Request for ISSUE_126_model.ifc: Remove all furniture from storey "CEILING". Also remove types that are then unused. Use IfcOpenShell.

First a look at what the model holds.

```python
import ifcopenshell
import ifcopenshell.util.element

model = ifcopenshell.open("ISSUE_126_model.ifc")
print(model.schema)
storey = next(s for s in model.by_type("IfcBuildingStorey") if s.Name == "CEILING")
furniture = [e for e in ifcopenshell.util.element.get_decomposition(storey) if e.is_a("IfcFurnishingElement")]
seen = {}
for e in furniture:
    element_type = ifcopenshell.util.element.get_type(e)
    name = element_type.Name if element_type not in (None, e) else None
    seen[name] = seen.get(name, 0) + 1
for name, count in sorted(seen.items(), key=str):
    print(count, "x", name)
```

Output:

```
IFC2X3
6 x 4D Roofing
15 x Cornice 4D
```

```python
import ifcopenshell
import ifcopenshell.api.root
import ifcopenshell.util.element

model = ifcopenshell.open("ISSUE_126_model.ifc")

storey = next(s for s in model.by_type("IfcBuildingStorey") if s.Name == "CEILING")
furniture = [e for e in ifcopenshell.util.element.get_decomposition(storey) if e.is_a("IfcFurnishingElement")]
types = {ifcopenshell.util.element.get_type(e) for e in furniture} - {None, *furniture}

for e in furniture:
    ifcopenshell.api.root.remove_product(model, product=e)
print(len(furniture), "removed")

unused = [t for t in types if not ifcopenshell.util.element.get_types(t)]
for t in unused:
    ifcopenshell.api.root.remove_product(model, product=t)
print(len(unused), "unused types removed")

model.write("ISSUE_126_model_edited.ifc")
```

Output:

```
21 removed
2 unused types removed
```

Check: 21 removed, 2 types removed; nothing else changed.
